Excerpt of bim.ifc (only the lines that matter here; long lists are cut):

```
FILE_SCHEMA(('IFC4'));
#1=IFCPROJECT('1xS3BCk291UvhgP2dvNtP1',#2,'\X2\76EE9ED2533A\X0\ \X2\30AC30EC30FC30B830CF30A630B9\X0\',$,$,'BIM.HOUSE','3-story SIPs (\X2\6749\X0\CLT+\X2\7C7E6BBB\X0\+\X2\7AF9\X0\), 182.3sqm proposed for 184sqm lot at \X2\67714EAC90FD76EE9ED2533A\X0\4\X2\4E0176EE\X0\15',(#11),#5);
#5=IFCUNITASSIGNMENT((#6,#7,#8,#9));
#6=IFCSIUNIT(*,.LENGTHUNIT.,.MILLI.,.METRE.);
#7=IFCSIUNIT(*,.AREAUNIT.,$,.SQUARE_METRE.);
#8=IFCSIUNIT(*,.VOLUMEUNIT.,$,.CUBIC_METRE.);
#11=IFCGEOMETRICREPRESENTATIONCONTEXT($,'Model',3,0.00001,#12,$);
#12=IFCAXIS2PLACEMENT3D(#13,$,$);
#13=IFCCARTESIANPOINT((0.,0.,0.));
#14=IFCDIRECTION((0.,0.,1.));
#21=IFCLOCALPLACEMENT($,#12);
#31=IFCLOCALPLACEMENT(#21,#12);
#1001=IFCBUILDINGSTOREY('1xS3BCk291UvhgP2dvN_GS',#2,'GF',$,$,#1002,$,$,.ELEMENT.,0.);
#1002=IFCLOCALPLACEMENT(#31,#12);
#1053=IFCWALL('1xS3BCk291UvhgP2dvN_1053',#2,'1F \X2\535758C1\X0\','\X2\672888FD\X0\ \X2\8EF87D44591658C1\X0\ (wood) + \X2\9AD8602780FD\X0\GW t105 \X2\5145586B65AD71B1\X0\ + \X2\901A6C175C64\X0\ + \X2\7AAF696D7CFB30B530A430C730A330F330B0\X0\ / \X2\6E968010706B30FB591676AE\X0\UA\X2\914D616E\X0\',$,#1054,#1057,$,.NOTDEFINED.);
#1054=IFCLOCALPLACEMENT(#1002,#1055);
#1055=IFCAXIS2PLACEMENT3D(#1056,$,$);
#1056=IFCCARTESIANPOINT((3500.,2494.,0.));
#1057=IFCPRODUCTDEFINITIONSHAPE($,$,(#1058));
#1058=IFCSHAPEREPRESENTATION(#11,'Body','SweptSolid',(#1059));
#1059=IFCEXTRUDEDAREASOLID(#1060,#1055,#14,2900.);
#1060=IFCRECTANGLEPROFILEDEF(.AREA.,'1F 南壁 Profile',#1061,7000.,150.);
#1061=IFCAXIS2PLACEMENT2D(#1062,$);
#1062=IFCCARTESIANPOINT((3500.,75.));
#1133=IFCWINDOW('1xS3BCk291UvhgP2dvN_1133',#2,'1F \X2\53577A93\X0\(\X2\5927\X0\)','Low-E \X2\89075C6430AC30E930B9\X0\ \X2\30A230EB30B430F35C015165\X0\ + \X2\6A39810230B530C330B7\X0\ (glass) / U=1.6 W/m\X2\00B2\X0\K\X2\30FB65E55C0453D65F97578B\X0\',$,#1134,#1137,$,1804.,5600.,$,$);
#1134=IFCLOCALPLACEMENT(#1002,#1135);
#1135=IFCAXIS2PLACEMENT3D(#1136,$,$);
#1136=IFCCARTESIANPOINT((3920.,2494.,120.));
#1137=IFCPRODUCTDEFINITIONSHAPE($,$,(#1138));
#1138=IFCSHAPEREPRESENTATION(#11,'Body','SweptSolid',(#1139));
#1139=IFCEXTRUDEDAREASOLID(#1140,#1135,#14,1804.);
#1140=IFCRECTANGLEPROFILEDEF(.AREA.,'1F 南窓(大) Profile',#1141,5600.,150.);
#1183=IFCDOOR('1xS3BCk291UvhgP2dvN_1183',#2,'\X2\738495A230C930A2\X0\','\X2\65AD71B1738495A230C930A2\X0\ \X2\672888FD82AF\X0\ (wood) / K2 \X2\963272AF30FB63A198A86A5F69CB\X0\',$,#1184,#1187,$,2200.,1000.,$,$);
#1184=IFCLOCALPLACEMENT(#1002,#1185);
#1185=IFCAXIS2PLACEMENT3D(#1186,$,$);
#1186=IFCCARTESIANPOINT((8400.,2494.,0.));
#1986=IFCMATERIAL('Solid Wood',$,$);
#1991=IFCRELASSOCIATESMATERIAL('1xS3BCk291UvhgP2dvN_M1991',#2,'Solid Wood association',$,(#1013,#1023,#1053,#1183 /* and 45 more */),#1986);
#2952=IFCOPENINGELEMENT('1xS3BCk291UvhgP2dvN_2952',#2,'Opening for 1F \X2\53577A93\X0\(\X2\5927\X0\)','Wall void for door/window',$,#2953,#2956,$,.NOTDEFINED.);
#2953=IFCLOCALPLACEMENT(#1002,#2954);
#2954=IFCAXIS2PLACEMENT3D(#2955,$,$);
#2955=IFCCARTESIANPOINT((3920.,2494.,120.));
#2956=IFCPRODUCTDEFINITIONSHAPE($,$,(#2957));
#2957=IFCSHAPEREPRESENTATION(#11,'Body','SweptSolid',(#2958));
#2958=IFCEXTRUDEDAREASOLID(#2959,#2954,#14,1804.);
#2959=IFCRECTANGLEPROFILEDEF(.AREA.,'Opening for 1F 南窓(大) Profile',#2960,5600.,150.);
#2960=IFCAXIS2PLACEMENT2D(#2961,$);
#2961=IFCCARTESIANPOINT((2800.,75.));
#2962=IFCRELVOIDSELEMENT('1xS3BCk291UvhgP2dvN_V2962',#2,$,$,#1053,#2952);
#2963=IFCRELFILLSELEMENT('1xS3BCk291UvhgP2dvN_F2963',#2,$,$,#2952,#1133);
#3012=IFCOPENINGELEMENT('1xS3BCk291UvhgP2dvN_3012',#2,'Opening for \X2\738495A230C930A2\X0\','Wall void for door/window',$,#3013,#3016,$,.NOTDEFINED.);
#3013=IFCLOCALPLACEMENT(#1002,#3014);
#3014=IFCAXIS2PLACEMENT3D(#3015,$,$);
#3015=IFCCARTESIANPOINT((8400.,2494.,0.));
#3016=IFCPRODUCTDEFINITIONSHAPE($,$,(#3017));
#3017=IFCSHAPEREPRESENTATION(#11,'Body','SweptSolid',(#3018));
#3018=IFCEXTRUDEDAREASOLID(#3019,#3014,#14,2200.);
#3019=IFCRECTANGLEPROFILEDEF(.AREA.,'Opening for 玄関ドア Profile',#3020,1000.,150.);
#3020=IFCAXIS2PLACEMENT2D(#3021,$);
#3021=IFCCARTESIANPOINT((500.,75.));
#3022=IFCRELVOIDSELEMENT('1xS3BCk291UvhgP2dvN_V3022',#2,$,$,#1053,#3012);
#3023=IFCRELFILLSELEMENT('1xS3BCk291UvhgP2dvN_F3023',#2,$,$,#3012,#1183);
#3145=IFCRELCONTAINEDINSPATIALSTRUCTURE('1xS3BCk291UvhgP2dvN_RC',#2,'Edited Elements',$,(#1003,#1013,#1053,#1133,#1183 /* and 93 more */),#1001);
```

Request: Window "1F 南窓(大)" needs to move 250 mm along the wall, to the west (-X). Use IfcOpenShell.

```python
import ifcopenshell
import ifcopenshell.api.geometry
import ifcopenshell.util.placement
import ifcopenshell.util.unit

model = ifcopenshell.open("bim.ifc")
unit_scale = ifcopenshell.util.unit.calculate_unit_scale(model)

window = model.by_id(1133)
opening = window.FillsVoids[0].RelatingOpeningElement
wall = opening.VoidsElements[0].RelatingBuildingElement

wall_matrix = ifcopenshell.util.placement.get_local_placement(wall.ObjectPlacement)
shift = wall_matrix[:3, 0] * -0.25 / unit_scale
before = ifcopenshell.util.placement.get_local_placement(window.ObjectPlacement)[:3, 3].copy()

# The window is not placed relative to its opening, so move both.
for product in (opening, window):
    matrix = ifcopenshell.util.placement.get_local_placement(product.ObjectPlacement)
    matrix[:3, 3] += shift
    ifcopenshell.api.geometry.edit_object_placement(model, product=product, matrix=matrix, is_si=False)

after = ifcopenshell.util.placement.get_local_placement(window.ObjectPlacement)[:3, 3]
print("window moved by", (after - before).round(3) + 0.0)

model.write("bim_updated.ifc")
```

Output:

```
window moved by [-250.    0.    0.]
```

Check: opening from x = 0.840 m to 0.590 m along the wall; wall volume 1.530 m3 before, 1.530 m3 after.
